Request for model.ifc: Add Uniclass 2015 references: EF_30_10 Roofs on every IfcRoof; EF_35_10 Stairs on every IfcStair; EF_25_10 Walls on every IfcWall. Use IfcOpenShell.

First a look at what the model holds.

```python
import ifcopenshell

model = ifcopenshell.open("model.ifc")
print(model.schema)
print("classifications:", [c.Name for c in model.by_type("IfcClassification")])
for ifc_class in ("IfcDoor", "IfcRoof", "IfcStair", "IfcWall", "IfcWindow"):
    print(ifc_class, len(model.by_type(ifc_class)))
```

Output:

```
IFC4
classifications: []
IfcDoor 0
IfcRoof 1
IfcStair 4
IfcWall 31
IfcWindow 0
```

```python
import ifcopenshell
import ifcopenshell.api.classification

model = ifcopenshell.open("model.ifc")

system = ifcopenshell.api.classification.add_classification(model, classification="Uniclass 2015")

codes = {
    "IfcRoof": ("EF_30_10", "Roofs"),
    "IfcStair": ("EF_35_10", "Stairs"),
    "IfcWall": ("EF_25_10", "Walls"),
}
for ifc_class, (code, name) in codes.items():
    products = model.by_type(ifc_class)
    ifcopenshell.api.classification.add_reference(
        model, products=products, classification=system, identification=code, name=name
    )
    print(code, len(products))

model.write("model_v2.ifc")
```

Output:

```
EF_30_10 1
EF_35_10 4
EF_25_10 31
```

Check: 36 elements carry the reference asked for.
